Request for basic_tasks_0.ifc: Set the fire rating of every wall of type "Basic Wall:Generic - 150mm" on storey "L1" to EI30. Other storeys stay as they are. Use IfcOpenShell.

First a look at what the model holds.

```python
import ifcopenshell
import ifcopenshell.util.element

model = ifcopenshell.open("basic_tasks_0.ifc")
print(model.schema)
storey = next(s for s in model.by_type("IfcBuildingStorey") if s.Name == "L1")
walls = [e for e in ifcopenshell.util.element.get_decomposition(storey) if e.is_a("IfcWall")]
seen = {}
for e in walls:
    element_type = ifcopenshell.util.element.get_type(e)
    key = (element_type.Name if element_type != e and element_type else None, ifcopenshell.util.element.get_pset(e, "Pset_WallCommon", "FireRating"))
    seen[key] = seen.get(key, 0) + 1
for (name, value), count in sorted(seen.items(), key=str):
    print(count, "x", name, "|", value)
```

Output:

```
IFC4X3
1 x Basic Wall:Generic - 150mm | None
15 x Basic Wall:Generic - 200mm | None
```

```python
import ifcopenshell
import ifcopenshell.api.pset
import ifcopenshell.util.element

model = ifcopenshell.open("basic_tasks_0.ifc")

storey = next(s for s in model.by_type("IfcBuildingStorey") if s.Name == "L1")
walls = [e for e in ifcopenshell.util.element.get_decomposition(storey) if e.is_a("IfcWall")]

count = 0
for e in walls:
    element_type = ifcopenshell.util.element.get_type(e)
    if element_type in (None, e) or element_type.Name != "Basic Wall:Generic - 150mm":
        continue
    # add_pset returns the element's existing set when there is one.
    pset = ifcopenshell.api.pset.add_pset(model, product=e, name="Pset_WallCommon")
    ifcopenshell.api.pset.edit_pset(model, pset=pset, properties={"FireRating": "EI30"})
    count += 1

print(count, "walls updated")

model.write("basic_tasks_0_edited.ifc")
```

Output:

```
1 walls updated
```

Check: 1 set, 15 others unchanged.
